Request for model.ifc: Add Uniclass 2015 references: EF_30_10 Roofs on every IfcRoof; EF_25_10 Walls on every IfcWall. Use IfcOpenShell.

First a look at what the model holds.

```python
import ifcopenshell

model = ifcopenshell.open("model.ifc")
print(model.schema)
print("classifications:", [c.Name for c in model.by_type("IfcClassification")])
for ifc_class in ("IfcDoor", "IfcRoof", "IfcStair", "IfcWall", "IfcWindow"):
    print(ifc_class, len(model.by_type(ifc_class)))
```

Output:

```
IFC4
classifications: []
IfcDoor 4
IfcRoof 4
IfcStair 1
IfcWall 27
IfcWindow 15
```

```python
import ifcopenshell
import ifcopenshell.api.classification

model = ifcopenshell.open("model.ifc")

system = ifcopenshell.api.classification.add_classification(model, classification="Uniclass 2015")

codes = {
    "IfcRoof": ("EF_30_10", "Roofs"),
    "IfcWall": ("EF_25_10", "Walls"),
}
for ifc_class, (code, name) in codes.items():
    products = model.by_type(ifc_class)
    ifcopenshell.api.classification.add_reference(
        model, products=products, classification=system, identification=code, name=name
    )
    print(code, len(products))

model.write("model-out.ifc")
```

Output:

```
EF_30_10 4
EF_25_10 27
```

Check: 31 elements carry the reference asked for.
